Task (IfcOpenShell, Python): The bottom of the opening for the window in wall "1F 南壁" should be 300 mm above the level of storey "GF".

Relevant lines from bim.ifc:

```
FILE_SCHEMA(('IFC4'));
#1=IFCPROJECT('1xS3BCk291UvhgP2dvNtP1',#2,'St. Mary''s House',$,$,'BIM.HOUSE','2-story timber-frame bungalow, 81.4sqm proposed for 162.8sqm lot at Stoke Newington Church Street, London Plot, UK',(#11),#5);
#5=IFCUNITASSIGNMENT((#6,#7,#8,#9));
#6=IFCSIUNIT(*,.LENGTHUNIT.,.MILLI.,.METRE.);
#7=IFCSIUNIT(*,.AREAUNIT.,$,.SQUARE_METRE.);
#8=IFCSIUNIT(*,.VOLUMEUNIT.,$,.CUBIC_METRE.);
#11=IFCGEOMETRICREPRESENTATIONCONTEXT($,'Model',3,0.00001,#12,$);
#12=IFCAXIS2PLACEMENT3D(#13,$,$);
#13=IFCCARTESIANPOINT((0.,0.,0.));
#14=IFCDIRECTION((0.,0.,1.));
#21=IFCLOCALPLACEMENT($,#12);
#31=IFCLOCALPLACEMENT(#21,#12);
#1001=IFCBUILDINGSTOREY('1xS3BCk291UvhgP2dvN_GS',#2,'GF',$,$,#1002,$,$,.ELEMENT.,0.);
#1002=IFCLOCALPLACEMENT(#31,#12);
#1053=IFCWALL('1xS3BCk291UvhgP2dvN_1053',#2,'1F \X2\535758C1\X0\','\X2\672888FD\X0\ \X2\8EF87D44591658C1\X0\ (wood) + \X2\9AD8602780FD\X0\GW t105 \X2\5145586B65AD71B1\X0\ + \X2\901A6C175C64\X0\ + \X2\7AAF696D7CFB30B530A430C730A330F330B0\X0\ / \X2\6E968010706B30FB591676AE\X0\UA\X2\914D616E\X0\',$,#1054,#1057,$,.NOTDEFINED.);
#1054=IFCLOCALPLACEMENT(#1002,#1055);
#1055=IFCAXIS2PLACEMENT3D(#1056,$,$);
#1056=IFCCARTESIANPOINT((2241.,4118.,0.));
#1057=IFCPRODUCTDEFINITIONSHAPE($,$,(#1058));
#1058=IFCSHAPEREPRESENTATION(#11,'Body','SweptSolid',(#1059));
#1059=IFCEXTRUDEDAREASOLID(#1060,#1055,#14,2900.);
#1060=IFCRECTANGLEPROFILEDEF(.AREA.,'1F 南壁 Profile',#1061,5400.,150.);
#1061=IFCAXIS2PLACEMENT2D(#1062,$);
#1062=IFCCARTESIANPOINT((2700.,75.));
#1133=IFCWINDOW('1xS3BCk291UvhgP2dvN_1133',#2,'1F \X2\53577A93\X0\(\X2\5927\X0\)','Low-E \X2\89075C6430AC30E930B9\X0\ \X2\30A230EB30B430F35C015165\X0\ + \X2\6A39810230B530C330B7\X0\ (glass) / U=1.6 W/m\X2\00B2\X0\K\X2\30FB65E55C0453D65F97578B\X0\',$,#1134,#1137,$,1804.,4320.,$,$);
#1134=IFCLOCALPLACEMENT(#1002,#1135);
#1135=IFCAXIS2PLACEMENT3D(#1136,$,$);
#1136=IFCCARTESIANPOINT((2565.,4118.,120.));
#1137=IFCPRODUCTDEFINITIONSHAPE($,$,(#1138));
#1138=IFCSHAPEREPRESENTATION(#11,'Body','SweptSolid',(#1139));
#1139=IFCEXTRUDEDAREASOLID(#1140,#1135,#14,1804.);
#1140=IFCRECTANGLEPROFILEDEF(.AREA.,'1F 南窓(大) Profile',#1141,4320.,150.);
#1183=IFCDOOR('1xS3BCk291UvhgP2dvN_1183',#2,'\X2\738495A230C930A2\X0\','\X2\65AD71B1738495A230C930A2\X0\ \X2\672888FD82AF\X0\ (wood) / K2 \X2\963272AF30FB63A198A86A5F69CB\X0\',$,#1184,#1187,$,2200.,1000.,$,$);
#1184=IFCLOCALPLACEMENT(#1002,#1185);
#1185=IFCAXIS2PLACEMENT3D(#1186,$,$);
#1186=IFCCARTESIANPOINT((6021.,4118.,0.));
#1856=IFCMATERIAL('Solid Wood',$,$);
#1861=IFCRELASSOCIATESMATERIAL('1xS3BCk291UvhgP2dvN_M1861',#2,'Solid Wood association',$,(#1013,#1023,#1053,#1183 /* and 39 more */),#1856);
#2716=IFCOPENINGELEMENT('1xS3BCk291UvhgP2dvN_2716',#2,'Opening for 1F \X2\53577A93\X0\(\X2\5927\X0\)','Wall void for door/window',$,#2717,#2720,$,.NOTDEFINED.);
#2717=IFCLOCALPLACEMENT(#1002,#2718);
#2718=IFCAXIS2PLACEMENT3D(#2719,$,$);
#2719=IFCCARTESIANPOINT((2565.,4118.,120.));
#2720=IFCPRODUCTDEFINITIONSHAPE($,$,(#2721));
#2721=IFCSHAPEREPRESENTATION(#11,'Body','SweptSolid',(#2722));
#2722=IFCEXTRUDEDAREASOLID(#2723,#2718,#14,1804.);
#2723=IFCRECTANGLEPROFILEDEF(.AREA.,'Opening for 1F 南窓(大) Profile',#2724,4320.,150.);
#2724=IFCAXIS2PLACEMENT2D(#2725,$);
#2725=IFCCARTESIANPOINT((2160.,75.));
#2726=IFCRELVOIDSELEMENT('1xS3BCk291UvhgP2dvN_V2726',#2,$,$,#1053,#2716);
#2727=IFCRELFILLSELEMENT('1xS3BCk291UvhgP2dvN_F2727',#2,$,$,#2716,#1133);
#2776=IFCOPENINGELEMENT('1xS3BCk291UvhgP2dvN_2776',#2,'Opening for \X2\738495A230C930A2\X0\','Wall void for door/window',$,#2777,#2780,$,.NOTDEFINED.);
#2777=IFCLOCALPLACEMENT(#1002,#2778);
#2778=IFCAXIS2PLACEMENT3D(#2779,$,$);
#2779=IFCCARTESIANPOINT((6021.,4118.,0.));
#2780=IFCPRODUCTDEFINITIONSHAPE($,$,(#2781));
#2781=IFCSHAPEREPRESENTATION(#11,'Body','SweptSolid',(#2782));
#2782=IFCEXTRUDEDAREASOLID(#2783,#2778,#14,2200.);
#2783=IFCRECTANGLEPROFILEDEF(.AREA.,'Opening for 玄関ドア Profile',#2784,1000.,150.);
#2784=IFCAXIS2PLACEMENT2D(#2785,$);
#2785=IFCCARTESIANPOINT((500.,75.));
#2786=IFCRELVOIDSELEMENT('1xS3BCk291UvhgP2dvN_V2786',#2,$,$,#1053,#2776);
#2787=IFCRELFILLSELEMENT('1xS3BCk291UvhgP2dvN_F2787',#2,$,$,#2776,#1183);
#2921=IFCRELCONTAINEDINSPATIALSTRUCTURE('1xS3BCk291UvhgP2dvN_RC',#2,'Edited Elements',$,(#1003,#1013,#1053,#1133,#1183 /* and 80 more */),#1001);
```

```python
import numpy as np
import ifcopenshell
import ifcopenshell.api.geometry
import ifcopenshell.geom
import ifcopenshell.util.element
import ifcopenshell.util.placement
import ifcopenshell.util.shape
import ifcopenshell.util.unit

model = ifcopenshell.open("bim.ifc")
unit_scale = ifcopenshell.util.unit.calculate_unit_scale(model)

window = model.by_id(1133)
opening = window.FillsVoids[0].RelatingOpeningElement
storey = ifcopenshell.util.element.get_container(window, ifc_class="IfcBuildingStorey")
level = ifcopenshell.util.placement.get_local_placement(storey.ObjectPlacement)[2, 3]

# The opening's origin need not be at the sill, so measure its lowest point.
shape = ifcopenshell.geom.create_shape(ifcopenshell.geom.settings(), opening)
bottom = ifcopenshell.util.shape.get_shape_bottom_elevation(shape, shape.geometry) / unit_scale
dz = level + 0.3 / unit_scale - bottom

shift = np.array([0.0, 0.0, dz])
# The window is not placed relative to its opening, so move both.
for product in (opening, window):
    matrix = ifcopenshell.util.placement.get_local_placement(product.ObjectPlacement)
    matrix[:3, 3] += shift
    ifcopenshell.api.geometry.edit_object_placement(model, product=product, matrix=matrix, is_si=False)

print(f"moved by {dz * unit_scale:+.3f} m")

model.write("bim_v2.ifc")
```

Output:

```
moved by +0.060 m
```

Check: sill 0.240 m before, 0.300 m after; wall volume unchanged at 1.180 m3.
